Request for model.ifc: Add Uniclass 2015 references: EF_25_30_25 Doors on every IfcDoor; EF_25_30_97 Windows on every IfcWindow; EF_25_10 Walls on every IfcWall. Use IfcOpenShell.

First a look at what the model holds.

```python
import ifcopenshell

model = ifcopenshell.open("model.ifc")
print(model.schema)
print("classifications:", [c.Name for c in model.by_type("IfcClassification")])
for ifc_class in ("IfcDoor", "IfcRoof", "IfcStair", "IfcWall", "IfcWindow"):
    print(ifc_class, len(model.by_type(ifc_class)))
```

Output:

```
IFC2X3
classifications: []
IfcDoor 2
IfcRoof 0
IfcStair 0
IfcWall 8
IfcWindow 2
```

```python
import ifcopenshell
import ifcopenshell.api.classification

model = ifcopenshell.open("model.ifc")

# IFC2X3 requires Source and Edition and has no link from the project to the system.
system = model.create_entity("IfcClassification", Source="NBS", Edition="2015", Name="Uniclass 2015")

codes = {
    "IfcDoor": ("EF_25_30_25", "Doors"),
    "IfcWindow": ("EF_25_30_97", "Windows"),
    "IfcWall": ("EF_25_10", "Walls"),
}
for ifc_class, (code, name) in codes.items():
    products = model.by_type(ifc_class)
    ifcopenshell.api.classification.add_reference(
        model, products=products, classification=system, identification=code, name=name
    )
    print(code, len(products))

model.write("model-out.ifc")
```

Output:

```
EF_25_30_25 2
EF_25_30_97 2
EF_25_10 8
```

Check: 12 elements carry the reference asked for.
